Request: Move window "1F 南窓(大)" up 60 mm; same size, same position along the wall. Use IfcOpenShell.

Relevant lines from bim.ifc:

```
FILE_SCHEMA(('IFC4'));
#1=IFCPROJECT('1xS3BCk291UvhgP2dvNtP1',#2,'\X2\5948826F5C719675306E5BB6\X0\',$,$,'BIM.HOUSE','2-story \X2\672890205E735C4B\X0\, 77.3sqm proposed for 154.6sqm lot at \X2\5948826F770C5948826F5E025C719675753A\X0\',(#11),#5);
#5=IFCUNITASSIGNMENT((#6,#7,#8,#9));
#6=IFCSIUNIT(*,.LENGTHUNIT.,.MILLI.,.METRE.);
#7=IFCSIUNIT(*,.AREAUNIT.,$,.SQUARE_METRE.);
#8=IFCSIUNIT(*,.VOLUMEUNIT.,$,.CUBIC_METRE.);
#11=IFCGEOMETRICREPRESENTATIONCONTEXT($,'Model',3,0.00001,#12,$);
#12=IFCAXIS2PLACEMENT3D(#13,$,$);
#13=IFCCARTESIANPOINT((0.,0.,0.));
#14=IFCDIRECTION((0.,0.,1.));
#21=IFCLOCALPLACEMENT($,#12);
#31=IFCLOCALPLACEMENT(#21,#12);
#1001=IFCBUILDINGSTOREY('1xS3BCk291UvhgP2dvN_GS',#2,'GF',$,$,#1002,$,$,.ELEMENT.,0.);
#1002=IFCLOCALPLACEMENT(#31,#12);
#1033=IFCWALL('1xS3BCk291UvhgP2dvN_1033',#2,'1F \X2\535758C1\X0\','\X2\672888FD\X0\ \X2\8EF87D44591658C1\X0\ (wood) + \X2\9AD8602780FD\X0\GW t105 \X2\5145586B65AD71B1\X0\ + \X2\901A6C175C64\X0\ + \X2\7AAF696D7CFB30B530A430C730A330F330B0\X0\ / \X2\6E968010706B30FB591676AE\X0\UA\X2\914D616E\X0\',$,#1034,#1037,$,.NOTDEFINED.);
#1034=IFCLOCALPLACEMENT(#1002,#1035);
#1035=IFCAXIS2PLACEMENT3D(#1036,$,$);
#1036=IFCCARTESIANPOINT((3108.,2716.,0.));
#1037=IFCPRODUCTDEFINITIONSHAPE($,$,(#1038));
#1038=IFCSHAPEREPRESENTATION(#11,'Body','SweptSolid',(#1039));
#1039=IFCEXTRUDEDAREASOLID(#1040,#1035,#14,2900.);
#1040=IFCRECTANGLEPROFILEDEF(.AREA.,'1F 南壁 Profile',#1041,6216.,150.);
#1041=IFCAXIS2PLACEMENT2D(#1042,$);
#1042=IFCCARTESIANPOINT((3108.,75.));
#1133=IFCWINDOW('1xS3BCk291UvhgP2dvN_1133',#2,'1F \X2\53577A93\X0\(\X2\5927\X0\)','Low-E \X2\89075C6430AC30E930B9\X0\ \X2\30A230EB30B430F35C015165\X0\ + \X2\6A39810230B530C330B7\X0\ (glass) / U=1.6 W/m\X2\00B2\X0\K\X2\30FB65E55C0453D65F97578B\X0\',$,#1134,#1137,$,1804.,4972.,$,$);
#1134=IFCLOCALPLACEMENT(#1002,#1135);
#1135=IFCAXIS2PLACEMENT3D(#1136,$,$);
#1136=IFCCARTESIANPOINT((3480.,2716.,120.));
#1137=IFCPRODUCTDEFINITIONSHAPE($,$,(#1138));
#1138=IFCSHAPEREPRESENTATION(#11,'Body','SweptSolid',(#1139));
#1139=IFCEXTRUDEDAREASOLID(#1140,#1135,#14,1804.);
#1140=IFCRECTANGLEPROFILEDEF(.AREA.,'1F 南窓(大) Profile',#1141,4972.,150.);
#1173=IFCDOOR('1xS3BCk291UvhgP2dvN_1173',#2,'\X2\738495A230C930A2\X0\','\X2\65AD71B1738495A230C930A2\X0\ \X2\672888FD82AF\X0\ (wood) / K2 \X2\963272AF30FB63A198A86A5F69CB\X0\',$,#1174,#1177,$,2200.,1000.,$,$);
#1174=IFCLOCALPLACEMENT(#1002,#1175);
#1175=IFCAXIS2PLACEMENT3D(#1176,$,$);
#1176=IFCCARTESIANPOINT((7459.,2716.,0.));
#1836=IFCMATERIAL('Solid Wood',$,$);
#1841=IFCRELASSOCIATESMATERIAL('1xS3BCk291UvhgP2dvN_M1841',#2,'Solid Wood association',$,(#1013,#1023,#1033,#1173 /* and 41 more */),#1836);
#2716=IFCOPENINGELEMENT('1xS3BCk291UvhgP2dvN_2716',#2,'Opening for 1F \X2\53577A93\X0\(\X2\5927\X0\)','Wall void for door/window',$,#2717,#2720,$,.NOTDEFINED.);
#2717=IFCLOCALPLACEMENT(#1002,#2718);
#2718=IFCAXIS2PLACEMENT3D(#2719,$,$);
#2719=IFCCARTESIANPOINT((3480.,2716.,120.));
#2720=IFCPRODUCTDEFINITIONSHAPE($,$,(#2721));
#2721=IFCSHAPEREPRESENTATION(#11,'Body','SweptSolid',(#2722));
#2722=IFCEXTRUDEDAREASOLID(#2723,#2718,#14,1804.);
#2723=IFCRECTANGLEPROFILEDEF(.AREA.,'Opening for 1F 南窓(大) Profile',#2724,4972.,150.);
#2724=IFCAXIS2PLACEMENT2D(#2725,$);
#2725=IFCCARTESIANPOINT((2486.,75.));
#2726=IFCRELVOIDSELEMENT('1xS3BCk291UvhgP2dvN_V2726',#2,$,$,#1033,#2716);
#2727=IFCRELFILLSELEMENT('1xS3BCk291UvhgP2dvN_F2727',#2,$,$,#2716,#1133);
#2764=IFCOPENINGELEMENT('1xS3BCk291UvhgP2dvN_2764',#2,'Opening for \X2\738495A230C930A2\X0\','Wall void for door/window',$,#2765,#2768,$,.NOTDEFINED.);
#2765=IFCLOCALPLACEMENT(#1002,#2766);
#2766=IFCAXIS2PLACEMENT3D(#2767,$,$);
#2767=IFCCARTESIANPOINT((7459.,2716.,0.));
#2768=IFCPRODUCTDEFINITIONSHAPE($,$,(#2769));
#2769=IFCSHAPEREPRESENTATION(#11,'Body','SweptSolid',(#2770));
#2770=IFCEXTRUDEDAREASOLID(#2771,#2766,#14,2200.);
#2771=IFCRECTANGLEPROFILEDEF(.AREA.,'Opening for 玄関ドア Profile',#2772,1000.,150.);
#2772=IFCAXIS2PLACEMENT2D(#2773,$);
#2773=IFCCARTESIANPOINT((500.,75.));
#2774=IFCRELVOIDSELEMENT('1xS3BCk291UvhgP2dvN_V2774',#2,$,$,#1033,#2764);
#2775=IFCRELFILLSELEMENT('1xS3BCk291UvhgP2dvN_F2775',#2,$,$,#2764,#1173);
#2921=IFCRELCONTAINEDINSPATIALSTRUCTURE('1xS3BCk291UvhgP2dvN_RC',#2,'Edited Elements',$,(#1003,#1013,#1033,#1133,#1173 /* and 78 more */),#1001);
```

```python
import numpy as np
import ifcopenshell
import ifcopenshell.api.geometry
import ifcopenshell.util.placement
import ifcopenshell.util.unit

model = ifcopenshell.open("bim.ifc")
unit_scale = ifcopenshell.util.unit.calculate_unit_scale(model)

window = model.by_id(1133)
opening = window.FillsVoids[0].RelatingOpeningElement
dz = 0.06 / unit_scale

shift = np.array([0.0, 0.0, dz])
# The window is not placed relative to its opening, so move both.
for product in (opening, window):
    matrix = ifcopenshell.util.placement.get_local_placement(product.ObjectPlacement)
    matrix[:3, 3] += shift
    ifcopenshell.api.geometry.edit_object_placement(model, product=product, matrix=matrix, is_si=False)

print(f"moved by {dz * unit_scale:+.3f} m")

model.write("bim_v2.ifc")
```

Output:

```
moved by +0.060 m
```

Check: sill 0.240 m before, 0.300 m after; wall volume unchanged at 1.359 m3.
